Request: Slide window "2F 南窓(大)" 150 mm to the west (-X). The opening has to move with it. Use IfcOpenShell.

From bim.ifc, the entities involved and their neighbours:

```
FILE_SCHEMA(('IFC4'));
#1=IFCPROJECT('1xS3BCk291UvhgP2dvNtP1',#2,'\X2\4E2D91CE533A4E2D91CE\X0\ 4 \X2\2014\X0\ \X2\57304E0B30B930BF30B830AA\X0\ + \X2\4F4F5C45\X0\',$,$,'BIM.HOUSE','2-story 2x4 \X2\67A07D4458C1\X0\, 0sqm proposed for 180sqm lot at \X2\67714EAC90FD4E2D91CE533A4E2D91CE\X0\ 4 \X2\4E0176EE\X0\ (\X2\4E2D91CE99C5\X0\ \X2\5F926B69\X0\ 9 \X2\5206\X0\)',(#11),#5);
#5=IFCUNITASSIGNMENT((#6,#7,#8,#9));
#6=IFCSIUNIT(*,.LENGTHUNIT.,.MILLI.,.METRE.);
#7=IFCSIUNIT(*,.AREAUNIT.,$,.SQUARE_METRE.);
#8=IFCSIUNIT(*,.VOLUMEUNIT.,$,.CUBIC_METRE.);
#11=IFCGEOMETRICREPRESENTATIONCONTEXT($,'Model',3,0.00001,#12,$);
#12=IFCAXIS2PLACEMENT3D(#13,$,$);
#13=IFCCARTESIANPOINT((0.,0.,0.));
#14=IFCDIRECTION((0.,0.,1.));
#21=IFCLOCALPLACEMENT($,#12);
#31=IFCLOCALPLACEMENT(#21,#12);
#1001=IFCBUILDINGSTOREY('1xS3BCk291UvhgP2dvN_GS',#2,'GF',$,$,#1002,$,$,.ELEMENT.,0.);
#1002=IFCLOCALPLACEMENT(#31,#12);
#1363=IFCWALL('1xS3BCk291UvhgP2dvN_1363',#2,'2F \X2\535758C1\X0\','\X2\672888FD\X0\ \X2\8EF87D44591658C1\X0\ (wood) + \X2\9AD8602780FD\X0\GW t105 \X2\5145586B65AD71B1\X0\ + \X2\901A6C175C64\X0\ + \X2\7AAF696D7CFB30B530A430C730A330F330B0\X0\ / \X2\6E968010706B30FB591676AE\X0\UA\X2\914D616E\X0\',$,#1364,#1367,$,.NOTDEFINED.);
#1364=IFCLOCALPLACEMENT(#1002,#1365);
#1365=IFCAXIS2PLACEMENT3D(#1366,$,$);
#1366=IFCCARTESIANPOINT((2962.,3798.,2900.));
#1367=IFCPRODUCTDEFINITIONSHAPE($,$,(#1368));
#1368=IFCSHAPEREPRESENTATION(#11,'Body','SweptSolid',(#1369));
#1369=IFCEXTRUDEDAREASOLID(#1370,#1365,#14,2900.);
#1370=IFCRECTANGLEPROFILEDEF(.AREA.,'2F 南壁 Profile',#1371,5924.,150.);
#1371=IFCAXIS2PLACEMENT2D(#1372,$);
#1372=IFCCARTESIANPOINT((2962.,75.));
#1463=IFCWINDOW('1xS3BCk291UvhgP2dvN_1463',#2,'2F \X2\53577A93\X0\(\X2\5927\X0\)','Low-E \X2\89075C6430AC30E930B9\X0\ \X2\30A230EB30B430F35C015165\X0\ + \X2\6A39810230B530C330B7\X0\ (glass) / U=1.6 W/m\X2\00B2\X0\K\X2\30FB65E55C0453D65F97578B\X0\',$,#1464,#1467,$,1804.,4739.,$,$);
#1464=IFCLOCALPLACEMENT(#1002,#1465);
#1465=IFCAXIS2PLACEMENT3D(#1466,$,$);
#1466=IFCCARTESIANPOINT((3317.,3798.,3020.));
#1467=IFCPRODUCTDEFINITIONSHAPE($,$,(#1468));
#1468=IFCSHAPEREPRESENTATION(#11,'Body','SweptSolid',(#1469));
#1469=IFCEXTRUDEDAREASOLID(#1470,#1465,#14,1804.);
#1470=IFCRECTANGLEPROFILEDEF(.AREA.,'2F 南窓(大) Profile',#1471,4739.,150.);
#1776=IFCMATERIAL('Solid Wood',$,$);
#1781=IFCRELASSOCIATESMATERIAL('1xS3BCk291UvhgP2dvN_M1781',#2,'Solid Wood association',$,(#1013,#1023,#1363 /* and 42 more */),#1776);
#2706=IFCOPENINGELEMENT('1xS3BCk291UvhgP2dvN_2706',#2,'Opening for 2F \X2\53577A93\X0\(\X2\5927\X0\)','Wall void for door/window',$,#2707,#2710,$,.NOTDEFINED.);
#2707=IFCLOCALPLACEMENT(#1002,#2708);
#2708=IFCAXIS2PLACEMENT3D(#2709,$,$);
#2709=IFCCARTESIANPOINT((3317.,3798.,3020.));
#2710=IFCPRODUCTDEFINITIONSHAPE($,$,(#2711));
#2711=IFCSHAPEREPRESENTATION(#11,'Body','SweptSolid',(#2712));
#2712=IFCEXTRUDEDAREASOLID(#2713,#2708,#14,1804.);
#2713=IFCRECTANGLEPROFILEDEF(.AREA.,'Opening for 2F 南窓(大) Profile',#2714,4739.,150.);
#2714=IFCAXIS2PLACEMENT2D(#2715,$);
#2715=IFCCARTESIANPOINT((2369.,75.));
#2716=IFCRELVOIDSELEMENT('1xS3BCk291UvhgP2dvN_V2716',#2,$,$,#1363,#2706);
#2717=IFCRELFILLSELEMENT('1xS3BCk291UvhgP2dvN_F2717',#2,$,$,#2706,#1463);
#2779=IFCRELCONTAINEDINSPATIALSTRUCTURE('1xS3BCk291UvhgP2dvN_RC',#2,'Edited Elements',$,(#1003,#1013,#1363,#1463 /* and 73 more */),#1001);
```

```python
import ifcopenshell
import ifcopenshell.api.geometry
import ifcopenshell.util.placement
import ifcopenshell.util.unit

model = ifcopenshell.open("bim.ifc")
unit_scale = ifcopenshell.util.unit.calculate_unit_scale(model)

window = model.by_guid("1xS3BCk291UvhgP2dvN_1463")
opening = window.FillsVoids[0].RelatingOpeningElement
wall = opening.VoidsElements[0].RelatingBuildingElement

wall_matrix = ifcopenshell.util.placement.get_local_placement(wall.ObjectPlacement)
shift = wall_matrix[:3, 0] * -0.15 / unit_scale
before = ifcopenshell.util.placement.get_local_placement(window.ObjectPlacement)[:3, 3].copy()

# The window is not placed relative to its opening, so move both.
for product in (opening, window):
    matrix = ifcopenshell.util.placement.get_local_placement(product.ObjectPlacement)
    matrix[:3, 3] += shift
    ifcopenshell.api.geometry.edit_object_placement(model, product=product, matrix=matrix, is_si=False)

after = ifcopenshell.util.placement.get_local_placement(window.ObjectPlacement)[:3, 3]
print("window moved by", (after - before).round(3) + 0.0)

model.write("bim_updated.ifc")
```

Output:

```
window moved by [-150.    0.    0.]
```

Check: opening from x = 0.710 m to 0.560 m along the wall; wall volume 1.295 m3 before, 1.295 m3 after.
